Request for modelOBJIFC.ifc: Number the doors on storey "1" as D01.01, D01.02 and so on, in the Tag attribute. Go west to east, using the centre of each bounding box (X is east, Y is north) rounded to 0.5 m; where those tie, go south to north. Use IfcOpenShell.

First a look at what the model holds.

```python
import ifcopenshell
import ifcopenshell.util.element
import ifcopenshell.util.placement

model = ifcopenshell.open("modelOBJIFC.ifc")
print(model.schema)
storey = next(s for s in model.by_type("IfcBuildingStorey") if s.Name == "1")
doors = [e for e in ifcopenshell.util.element.get_decomposition(storey) if e.is_a("IfcDoor")]
for e in sorted(doors, key=lambda e: e.id()):
    origin = ifcopenshell.util.placement.get_local_placement(e.ObjectPlacement)[:3, 3]
    print(e.id(), e.Tag, e.Name, origin.round(2) + 0.0, sep=" | ")
```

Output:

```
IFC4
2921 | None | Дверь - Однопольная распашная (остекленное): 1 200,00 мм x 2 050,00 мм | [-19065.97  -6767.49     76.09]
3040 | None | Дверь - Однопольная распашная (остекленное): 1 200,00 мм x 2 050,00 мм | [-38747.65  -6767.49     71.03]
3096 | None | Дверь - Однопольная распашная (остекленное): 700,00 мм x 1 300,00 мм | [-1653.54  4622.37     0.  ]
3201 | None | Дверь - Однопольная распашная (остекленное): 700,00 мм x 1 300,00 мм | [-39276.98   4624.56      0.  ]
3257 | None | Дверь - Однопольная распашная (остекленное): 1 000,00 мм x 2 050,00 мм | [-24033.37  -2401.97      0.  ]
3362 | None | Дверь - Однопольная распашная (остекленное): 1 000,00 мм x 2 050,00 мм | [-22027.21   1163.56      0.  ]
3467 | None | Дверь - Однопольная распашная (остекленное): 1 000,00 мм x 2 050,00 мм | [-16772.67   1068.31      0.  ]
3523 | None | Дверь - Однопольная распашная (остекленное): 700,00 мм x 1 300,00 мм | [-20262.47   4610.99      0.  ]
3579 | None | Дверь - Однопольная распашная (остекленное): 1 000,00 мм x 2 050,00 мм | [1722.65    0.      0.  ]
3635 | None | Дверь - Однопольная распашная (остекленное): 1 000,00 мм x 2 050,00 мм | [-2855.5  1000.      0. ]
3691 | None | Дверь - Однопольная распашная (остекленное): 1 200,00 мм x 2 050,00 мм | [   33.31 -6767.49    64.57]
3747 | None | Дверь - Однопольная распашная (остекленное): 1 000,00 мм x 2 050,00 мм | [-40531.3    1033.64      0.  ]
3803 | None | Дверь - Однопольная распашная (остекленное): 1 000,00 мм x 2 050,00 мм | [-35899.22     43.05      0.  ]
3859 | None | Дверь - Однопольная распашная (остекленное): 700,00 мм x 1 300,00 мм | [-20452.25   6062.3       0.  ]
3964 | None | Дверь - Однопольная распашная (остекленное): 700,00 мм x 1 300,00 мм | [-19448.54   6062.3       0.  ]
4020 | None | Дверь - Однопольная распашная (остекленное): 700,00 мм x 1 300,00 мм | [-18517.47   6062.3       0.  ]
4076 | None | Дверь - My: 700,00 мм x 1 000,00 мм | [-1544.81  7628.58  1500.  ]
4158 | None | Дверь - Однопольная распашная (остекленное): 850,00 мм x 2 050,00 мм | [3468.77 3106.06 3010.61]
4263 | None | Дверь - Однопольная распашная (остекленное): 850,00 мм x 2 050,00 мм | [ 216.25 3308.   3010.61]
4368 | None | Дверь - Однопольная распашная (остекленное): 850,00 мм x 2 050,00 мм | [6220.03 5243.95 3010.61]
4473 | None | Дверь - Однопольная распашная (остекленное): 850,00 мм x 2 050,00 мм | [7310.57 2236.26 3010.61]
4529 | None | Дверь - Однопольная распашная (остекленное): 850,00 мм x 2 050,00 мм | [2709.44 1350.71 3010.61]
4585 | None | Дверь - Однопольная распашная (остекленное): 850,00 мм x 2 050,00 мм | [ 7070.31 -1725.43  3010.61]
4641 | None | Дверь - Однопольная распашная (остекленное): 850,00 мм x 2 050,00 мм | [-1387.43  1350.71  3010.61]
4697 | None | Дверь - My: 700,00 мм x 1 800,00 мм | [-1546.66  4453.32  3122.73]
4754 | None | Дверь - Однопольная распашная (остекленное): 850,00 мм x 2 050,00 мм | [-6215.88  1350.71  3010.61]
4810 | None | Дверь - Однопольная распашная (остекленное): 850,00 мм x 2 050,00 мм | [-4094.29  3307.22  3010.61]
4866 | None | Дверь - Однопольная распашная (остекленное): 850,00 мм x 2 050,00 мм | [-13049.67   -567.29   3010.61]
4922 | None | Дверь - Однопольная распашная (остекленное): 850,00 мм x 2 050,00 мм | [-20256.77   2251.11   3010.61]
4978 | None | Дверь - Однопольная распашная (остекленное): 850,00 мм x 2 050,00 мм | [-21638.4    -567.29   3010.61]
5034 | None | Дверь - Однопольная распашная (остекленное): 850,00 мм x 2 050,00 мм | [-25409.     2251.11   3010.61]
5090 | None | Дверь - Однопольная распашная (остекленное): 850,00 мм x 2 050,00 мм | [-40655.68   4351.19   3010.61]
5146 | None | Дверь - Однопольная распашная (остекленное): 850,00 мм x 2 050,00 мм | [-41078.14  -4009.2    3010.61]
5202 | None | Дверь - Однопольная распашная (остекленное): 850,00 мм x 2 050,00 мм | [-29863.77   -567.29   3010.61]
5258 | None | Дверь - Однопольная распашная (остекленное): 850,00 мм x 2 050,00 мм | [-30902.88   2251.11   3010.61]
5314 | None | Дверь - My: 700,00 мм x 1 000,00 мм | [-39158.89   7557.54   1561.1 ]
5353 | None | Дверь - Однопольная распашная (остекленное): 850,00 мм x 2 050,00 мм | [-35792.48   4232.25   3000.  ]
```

```python
import ifcopenshell
import ifcopenshell.geom
import ifcopenshell.util.element
import ifcopenshell.util.shape

model = ifcopenshell.open("modelOBJIFC.ifc")
settings = ifcopenshell.geom.settings()
settings.set("use-world-coords", True)


def centre(element):
    shape = ifcopenshell.geom.create_shape(settings, element)
    return ifcopenshell.util.shape.get_bbox_centroid(shape.geometry)


storey = next(s for s in model.by_type("IfcBuildingStorey") if s.Name == "1")
doors = [e for e in ifcopenshell.util.element.get_decomposition(storey) if e.is_a("IfcDoor")]

# Insertion points can sit at a corner or the storey origin, so sort by the geometry (in metres).
centres = {e: centre(e) for e in doors}
doors.sort(key=lambda e: (round(centres[e][0] / 0.5), centres[e][1]))

for i, e in enumerate(doors, start=1):
    number = f"D01.{i:02d}"
    e.Tag = number
    print(e.id(), number)

model.write("modelOBJIFC-out.ifc")
```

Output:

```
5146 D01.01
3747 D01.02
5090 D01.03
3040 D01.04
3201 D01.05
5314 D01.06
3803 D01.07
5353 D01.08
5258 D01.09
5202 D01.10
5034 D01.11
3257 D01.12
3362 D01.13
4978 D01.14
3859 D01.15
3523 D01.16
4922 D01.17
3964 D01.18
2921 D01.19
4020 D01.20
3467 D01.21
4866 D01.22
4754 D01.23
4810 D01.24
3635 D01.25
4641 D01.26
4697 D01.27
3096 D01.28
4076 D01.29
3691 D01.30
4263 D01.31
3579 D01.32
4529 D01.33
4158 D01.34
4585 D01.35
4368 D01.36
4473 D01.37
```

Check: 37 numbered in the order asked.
